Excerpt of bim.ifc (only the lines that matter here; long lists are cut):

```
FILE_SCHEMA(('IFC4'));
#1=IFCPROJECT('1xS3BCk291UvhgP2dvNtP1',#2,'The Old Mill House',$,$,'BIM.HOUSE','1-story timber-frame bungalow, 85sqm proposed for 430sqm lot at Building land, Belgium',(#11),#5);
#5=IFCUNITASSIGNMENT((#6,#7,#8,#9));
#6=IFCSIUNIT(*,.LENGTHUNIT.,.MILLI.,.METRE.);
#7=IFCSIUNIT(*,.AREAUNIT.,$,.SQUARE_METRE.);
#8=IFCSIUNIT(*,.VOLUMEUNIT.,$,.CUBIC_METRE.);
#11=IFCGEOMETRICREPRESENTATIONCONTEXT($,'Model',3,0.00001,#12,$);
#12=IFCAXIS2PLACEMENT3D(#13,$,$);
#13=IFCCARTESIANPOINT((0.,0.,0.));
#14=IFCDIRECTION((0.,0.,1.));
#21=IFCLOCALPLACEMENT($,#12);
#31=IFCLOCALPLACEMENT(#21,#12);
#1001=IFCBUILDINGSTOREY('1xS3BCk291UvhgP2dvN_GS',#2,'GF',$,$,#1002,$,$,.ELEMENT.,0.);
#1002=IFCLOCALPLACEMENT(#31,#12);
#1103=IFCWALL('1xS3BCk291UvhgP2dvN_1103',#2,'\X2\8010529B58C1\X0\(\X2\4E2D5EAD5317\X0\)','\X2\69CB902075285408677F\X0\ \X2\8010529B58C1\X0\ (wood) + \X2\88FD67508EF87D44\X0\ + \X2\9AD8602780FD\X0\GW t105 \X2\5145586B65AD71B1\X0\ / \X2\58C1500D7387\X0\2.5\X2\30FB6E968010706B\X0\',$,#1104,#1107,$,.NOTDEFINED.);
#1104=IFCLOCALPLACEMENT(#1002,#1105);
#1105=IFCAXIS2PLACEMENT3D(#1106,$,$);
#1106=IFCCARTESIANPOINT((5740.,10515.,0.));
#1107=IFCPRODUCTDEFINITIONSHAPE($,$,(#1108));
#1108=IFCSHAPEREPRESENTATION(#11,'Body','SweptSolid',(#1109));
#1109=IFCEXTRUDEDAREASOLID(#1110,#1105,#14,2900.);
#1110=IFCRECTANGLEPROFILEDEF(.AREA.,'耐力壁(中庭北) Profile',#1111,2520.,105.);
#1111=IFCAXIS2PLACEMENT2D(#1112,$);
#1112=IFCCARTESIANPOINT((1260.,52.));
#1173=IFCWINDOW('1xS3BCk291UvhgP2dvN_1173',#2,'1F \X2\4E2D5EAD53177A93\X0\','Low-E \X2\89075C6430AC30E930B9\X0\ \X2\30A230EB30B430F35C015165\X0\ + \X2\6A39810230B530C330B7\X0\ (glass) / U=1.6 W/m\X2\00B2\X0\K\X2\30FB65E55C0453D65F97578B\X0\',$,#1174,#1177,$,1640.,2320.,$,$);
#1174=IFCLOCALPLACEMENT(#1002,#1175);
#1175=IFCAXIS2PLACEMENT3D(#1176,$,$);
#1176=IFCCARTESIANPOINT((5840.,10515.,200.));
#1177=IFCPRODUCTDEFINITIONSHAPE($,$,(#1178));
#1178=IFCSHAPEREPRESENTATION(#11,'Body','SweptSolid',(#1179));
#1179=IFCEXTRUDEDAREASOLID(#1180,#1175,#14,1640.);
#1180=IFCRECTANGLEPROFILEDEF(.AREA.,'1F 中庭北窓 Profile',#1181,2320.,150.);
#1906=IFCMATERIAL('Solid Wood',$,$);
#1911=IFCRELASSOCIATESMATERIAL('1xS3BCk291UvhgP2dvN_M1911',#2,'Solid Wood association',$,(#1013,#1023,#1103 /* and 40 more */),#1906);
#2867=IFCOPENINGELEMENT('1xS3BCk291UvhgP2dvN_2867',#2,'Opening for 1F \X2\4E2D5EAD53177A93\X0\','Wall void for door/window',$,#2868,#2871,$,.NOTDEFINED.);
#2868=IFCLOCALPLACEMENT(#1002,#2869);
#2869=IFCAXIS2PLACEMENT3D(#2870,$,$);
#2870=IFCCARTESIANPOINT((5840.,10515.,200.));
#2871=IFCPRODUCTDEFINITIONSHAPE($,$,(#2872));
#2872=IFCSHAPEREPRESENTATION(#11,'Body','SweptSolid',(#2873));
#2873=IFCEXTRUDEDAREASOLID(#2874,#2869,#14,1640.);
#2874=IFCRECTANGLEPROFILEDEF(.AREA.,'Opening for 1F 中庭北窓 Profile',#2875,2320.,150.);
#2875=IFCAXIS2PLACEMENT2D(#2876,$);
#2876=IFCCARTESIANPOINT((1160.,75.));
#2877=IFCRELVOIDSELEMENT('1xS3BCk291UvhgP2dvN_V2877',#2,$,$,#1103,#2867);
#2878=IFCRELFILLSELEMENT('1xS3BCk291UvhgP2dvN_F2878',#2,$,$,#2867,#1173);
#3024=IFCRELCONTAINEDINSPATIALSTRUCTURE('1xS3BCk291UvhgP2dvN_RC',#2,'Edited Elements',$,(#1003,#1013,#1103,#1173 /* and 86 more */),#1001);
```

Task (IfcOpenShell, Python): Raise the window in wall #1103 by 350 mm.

```python
import numpy as np
import ifcopenshell
import ifcopenshell.api.geometry
import ifcopenshell.util.placement
import ifcopenshell.util.unit

model = ifcopenshell.open("bim.ifc")
unit_scale = ifcopenshell.util.unit.calculate_unit_scale(model)

window = model.by_guid("1xS3BCk291UvhgP2dvN_1173")
opening = window.FillsVoids[0].RelatingOpeningElement
dz = 350.0

shift = np.array([0.0, 0.0, dz])
# The window is not placed relative to its opening, so move both.
for product in (opening, window):
    matrix = ifcopenshell.util.placement.get_local_placement(product.ObjectPlacement)
    matrix[:3, 3] += shift
    ifcopenshell.api.geometry.edit_object_placement(model, product=product, matrix=matrix, is_si=False)

print(f"moved by {dz * unit_scale:+.3f} m")

model.write("bim-out.ifc")
```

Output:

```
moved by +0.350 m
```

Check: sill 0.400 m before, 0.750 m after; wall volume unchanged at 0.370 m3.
